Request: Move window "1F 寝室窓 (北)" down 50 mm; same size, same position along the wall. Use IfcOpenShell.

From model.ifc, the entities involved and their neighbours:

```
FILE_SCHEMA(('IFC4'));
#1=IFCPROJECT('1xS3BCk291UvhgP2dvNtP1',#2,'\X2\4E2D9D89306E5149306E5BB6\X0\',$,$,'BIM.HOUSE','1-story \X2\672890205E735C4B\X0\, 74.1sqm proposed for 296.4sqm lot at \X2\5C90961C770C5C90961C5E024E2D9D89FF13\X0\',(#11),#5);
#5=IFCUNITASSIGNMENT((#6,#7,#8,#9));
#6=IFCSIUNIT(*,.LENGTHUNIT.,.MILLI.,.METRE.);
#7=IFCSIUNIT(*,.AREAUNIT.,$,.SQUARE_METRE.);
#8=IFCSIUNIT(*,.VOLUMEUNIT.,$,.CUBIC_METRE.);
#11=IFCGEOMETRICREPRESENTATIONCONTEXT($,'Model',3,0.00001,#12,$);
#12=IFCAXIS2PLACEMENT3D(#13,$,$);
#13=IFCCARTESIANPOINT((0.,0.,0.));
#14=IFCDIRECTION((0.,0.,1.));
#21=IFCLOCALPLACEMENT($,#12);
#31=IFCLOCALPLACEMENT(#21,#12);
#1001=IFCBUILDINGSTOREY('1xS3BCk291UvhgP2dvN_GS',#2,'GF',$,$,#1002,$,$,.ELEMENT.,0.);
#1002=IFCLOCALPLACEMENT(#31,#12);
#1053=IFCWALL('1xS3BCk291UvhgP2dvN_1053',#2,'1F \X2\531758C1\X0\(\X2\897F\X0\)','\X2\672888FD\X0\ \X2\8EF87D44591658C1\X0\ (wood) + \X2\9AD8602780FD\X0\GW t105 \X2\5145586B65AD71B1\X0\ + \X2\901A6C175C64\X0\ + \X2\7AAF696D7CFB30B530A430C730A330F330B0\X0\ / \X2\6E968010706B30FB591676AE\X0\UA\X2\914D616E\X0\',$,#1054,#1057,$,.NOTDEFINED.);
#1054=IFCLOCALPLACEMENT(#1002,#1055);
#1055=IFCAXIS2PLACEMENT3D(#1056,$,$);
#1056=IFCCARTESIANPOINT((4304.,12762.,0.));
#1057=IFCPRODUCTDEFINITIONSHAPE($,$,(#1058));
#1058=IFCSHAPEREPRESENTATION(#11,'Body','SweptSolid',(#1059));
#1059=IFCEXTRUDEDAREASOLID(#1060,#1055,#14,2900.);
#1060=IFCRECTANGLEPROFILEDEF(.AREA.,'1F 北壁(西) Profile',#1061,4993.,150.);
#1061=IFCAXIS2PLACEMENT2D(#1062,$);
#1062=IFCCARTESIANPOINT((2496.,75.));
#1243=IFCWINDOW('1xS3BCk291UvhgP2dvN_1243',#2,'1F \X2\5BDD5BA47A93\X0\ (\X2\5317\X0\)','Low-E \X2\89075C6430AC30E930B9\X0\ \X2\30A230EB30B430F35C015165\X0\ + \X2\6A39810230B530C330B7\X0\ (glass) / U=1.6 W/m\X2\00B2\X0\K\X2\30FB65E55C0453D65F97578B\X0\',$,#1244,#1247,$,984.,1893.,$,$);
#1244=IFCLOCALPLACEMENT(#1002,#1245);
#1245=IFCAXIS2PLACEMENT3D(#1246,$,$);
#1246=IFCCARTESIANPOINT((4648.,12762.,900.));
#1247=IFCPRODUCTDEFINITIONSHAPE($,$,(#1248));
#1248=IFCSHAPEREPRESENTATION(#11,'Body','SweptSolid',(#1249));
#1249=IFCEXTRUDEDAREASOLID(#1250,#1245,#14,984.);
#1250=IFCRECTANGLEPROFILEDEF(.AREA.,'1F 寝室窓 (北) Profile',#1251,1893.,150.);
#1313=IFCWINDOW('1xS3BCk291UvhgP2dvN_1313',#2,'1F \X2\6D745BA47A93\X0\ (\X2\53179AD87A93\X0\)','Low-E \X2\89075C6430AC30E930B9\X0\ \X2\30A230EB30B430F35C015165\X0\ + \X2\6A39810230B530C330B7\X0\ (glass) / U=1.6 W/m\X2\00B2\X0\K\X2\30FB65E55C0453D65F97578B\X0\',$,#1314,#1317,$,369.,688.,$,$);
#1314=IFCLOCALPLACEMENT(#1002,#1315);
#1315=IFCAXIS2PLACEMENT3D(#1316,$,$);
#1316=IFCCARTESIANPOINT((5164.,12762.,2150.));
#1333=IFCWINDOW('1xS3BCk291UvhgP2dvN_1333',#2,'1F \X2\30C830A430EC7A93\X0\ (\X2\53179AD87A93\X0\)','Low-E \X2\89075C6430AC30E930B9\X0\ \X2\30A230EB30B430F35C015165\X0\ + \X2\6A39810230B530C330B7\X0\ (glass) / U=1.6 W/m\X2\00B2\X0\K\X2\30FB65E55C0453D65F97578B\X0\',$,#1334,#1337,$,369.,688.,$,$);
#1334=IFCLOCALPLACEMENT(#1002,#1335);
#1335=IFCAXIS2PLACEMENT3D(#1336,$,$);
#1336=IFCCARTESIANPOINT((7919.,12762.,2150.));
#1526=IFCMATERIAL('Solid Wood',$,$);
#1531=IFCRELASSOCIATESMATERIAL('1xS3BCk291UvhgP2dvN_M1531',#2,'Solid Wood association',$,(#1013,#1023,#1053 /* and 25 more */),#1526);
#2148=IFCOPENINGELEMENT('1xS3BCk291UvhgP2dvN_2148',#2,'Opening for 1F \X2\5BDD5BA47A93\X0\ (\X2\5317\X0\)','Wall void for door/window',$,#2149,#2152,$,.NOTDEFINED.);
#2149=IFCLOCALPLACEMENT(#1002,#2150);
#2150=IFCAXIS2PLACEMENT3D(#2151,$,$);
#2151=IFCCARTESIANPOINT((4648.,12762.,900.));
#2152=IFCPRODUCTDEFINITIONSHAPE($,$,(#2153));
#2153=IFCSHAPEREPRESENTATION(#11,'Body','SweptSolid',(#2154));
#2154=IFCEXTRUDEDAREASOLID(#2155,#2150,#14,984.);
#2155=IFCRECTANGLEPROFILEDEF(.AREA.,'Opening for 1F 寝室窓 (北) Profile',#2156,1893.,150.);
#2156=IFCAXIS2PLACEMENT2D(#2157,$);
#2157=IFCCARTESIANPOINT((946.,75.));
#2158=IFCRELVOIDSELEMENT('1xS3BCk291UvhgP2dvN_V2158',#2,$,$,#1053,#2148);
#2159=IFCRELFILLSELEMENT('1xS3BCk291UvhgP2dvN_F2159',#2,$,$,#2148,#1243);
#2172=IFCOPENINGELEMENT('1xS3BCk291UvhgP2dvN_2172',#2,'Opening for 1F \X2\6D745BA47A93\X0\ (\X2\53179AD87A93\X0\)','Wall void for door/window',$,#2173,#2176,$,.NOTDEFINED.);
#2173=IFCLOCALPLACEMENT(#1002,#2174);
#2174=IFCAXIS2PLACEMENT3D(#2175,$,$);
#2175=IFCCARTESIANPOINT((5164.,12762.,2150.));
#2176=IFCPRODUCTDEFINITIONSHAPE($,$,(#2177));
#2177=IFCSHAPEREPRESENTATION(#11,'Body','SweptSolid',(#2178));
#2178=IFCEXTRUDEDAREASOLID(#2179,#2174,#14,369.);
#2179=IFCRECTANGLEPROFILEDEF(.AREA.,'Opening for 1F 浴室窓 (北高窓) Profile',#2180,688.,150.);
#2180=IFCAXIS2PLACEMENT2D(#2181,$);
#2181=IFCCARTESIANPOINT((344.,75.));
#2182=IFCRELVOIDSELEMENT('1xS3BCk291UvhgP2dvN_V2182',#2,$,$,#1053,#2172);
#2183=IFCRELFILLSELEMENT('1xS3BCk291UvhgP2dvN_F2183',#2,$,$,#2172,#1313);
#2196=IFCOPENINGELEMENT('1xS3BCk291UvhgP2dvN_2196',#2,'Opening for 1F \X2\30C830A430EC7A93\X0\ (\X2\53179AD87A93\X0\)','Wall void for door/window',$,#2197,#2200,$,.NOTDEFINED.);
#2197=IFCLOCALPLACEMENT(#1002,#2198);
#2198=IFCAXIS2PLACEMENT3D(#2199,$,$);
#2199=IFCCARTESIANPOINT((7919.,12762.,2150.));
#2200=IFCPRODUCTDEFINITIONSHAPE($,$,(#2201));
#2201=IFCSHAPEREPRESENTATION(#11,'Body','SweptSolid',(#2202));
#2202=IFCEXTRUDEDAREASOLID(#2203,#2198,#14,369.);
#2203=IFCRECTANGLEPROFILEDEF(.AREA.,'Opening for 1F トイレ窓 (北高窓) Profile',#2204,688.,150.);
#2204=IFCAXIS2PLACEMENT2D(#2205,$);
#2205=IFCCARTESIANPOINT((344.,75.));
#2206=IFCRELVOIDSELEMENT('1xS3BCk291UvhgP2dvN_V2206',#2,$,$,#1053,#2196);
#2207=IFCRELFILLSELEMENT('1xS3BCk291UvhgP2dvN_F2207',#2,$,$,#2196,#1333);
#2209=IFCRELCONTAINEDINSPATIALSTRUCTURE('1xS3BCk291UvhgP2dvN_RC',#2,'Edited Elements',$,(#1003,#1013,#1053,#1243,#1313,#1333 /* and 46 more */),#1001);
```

```python
import numpy as np
import ifcopenshell
import ifcopenshell.api.geometry
import ifcopenshell.util.placement
import ifcopenshell.util.unit

model = ifcopenshell.open("model.ifc")
unit_scale = ifcopenshell.util.unit.calculate_unit_scale(model)

window = model.by_guid("1xS3BCk291UvhgP2dvN_1243")
opening = window.FillsVoids[0].RelatingOpeningElement
dz = -50.0

shift = np.array([0.0, 0.0, dz])
# The window is not placed relative to its opening, so move both.
for product in (opening, window):
    matrix = ifcopenshell.util.placement.get_local_placement(product.ObjectPlacement)
    matrix[:3, 3] += shift
    ifcopenshell.api.geometry.edit_object_placement(model, product=product, matrix=matrix, is_si=False)

print(f"moved by {dz * unit_scale:+.3f} m")

model.write("model-out.ifc")
```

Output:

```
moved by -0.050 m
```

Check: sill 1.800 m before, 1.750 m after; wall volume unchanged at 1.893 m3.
